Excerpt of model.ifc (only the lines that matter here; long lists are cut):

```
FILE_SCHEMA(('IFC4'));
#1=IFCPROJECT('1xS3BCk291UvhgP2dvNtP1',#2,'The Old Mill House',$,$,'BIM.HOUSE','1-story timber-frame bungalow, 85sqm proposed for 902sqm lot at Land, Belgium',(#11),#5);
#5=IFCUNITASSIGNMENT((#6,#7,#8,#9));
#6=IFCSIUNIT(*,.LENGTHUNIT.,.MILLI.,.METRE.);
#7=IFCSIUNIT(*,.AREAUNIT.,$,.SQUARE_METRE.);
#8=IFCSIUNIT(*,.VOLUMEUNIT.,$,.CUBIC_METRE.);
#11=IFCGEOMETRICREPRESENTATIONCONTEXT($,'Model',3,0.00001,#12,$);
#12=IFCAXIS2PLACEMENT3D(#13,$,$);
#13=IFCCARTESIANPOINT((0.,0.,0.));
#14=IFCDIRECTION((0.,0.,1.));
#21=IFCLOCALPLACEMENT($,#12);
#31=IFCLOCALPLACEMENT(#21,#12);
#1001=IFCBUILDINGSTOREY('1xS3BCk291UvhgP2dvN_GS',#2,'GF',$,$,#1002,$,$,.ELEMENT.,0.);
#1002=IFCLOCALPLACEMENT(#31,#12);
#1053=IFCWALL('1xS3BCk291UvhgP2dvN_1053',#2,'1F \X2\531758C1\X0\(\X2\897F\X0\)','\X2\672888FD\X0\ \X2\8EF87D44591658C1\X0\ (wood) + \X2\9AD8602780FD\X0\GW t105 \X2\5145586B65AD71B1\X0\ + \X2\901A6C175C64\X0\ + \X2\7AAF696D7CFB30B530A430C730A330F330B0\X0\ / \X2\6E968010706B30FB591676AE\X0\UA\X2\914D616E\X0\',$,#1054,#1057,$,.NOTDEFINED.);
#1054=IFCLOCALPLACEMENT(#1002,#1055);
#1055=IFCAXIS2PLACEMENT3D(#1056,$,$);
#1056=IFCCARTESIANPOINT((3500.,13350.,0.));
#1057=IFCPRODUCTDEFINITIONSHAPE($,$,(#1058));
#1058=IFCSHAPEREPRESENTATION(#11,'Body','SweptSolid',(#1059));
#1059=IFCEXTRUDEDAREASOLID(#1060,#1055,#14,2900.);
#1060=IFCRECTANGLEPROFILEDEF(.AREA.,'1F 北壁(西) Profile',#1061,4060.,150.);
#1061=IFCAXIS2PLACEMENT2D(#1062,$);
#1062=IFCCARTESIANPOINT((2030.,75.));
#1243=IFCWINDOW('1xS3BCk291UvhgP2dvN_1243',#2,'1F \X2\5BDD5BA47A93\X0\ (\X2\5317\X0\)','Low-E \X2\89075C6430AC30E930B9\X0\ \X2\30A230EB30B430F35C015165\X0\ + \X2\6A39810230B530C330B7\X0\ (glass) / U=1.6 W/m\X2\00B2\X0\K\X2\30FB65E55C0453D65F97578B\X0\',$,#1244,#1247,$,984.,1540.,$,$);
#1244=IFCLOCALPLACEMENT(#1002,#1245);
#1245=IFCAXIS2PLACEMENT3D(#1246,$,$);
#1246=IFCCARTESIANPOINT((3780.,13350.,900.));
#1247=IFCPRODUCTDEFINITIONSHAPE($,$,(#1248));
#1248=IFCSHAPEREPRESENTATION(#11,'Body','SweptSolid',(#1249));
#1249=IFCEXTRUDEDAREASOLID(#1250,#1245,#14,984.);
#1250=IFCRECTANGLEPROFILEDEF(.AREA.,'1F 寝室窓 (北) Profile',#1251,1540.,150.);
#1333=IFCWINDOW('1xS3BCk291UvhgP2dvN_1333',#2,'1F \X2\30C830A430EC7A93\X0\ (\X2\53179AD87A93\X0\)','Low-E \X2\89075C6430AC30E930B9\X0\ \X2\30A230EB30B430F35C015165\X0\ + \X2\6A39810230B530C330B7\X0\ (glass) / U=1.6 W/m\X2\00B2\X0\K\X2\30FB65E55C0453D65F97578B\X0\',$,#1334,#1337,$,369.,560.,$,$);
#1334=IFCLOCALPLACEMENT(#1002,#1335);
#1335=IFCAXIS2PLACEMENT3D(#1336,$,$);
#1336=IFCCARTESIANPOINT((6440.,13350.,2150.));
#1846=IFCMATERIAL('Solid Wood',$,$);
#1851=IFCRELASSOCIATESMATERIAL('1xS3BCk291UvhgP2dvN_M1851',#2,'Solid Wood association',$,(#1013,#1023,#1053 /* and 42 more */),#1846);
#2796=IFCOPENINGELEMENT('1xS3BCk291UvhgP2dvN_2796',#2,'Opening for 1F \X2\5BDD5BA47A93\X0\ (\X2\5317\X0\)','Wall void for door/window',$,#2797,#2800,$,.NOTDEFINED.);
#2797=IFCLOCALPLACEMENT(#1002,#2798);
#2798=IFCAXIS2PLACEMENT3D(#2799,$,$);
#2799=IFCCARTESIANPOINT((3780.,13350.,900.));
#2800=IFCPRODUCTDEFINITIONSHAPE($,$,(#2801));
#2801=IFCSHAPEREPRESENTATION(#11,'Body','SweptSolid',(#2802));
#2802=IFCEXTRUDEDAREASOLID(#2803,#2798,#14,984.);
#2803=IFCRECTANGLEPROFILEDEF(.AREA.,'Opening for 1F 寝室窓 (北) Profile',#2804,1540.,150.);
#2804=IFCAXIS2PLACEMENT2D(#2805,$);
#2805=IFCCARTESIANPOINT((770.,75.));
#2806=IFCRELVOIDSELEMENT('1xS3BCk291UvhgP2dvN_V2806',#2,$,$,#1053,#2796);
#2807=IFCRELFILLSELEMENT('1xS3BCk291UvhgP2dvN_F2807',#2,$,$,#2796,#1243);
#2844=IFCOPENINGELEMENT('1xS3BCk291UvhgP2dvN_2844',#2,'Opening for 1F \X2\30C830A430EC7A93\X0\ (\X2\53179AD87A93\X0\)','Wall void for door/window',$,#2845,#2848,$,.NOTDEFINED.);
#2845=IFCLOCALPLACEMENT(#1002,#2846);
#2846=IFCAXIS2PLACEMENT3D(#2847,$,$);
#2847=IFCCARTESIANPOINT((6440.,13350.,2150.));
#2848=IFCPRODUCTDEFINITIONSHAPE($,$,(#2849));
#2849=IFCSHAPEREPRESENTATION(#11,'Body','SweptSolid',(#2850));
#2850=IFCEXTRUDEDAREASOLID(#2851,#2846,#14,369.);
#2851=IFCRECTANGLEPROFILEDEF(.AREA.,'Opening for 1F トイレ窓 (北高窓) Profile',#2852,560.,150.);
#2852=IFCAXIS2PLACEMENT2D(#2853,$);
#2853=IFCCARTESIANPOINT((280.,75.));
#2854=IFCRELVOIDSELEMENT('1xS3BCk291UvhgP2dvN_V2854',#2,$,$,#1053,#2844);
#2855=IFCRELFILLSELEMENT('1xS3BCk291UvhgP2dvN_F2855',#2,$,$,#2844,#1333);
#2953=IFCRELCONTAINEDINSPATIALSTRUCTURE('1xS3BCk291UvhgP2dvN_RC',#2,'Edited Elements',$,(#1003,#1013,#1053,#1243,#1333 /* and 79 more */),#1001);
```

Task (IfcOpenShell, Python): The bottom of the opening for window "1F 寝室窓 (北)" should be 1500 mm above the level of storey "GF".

```python
import numpy as np
import ifcopenshell
import ifcopenshell.api.geometry
import ifcopenshell.geom
import ifcopenshell.util.element
import ifcopenshell.util.placement
import ifcopenshell.util.shape
import ifcopenshell.util.unit

model = ifcopenshell.open("model.ifc")
unit_scale = ifcopenshell.util.unit.calculate_unit_scale(model)

window = model.by_id(1243)
opening = window.FillsVoids[0].RelatingOpeningElement
storey = ifcopenshell.util.element.get_container(window, ifc_class="IfcBuildingStorey")
level = ifcopenshell.util.placement.get_local_placement(storey.ObjectPlacement)[2, 3]

# The opening's origin need not be at the sill, so measure its lowest point.
shape = ifcopenshell.geom.create_shape(ifcopenshell.geom.settings(), opening)
bottom = ifcopenshell.util.shape.get_shape_bottom_elevation(shape, shape.geometry) / unit_scale
dz = level + 1.5 / unit_scale - bottom

shift = np.array([0.0, 0.0, dz])
# The window is not placed relative to its opening, so move both.
for product in (opening, window):
    matrix = ifcopenshell.util.placement.get_local_placement(product.ObjectPlacement)
    matrix[:3, 3] += shift
    ifcopenshell.api.geometry.edit_object_placement(model, product=product, matrix=matrix, is_si=False)

print(f"moved by {dz * unit_scale:+.3f} m")

model.write("model_v2.ifc")
```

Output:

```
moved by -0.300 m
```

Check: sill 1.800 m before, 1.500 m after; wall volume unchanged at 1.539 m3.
